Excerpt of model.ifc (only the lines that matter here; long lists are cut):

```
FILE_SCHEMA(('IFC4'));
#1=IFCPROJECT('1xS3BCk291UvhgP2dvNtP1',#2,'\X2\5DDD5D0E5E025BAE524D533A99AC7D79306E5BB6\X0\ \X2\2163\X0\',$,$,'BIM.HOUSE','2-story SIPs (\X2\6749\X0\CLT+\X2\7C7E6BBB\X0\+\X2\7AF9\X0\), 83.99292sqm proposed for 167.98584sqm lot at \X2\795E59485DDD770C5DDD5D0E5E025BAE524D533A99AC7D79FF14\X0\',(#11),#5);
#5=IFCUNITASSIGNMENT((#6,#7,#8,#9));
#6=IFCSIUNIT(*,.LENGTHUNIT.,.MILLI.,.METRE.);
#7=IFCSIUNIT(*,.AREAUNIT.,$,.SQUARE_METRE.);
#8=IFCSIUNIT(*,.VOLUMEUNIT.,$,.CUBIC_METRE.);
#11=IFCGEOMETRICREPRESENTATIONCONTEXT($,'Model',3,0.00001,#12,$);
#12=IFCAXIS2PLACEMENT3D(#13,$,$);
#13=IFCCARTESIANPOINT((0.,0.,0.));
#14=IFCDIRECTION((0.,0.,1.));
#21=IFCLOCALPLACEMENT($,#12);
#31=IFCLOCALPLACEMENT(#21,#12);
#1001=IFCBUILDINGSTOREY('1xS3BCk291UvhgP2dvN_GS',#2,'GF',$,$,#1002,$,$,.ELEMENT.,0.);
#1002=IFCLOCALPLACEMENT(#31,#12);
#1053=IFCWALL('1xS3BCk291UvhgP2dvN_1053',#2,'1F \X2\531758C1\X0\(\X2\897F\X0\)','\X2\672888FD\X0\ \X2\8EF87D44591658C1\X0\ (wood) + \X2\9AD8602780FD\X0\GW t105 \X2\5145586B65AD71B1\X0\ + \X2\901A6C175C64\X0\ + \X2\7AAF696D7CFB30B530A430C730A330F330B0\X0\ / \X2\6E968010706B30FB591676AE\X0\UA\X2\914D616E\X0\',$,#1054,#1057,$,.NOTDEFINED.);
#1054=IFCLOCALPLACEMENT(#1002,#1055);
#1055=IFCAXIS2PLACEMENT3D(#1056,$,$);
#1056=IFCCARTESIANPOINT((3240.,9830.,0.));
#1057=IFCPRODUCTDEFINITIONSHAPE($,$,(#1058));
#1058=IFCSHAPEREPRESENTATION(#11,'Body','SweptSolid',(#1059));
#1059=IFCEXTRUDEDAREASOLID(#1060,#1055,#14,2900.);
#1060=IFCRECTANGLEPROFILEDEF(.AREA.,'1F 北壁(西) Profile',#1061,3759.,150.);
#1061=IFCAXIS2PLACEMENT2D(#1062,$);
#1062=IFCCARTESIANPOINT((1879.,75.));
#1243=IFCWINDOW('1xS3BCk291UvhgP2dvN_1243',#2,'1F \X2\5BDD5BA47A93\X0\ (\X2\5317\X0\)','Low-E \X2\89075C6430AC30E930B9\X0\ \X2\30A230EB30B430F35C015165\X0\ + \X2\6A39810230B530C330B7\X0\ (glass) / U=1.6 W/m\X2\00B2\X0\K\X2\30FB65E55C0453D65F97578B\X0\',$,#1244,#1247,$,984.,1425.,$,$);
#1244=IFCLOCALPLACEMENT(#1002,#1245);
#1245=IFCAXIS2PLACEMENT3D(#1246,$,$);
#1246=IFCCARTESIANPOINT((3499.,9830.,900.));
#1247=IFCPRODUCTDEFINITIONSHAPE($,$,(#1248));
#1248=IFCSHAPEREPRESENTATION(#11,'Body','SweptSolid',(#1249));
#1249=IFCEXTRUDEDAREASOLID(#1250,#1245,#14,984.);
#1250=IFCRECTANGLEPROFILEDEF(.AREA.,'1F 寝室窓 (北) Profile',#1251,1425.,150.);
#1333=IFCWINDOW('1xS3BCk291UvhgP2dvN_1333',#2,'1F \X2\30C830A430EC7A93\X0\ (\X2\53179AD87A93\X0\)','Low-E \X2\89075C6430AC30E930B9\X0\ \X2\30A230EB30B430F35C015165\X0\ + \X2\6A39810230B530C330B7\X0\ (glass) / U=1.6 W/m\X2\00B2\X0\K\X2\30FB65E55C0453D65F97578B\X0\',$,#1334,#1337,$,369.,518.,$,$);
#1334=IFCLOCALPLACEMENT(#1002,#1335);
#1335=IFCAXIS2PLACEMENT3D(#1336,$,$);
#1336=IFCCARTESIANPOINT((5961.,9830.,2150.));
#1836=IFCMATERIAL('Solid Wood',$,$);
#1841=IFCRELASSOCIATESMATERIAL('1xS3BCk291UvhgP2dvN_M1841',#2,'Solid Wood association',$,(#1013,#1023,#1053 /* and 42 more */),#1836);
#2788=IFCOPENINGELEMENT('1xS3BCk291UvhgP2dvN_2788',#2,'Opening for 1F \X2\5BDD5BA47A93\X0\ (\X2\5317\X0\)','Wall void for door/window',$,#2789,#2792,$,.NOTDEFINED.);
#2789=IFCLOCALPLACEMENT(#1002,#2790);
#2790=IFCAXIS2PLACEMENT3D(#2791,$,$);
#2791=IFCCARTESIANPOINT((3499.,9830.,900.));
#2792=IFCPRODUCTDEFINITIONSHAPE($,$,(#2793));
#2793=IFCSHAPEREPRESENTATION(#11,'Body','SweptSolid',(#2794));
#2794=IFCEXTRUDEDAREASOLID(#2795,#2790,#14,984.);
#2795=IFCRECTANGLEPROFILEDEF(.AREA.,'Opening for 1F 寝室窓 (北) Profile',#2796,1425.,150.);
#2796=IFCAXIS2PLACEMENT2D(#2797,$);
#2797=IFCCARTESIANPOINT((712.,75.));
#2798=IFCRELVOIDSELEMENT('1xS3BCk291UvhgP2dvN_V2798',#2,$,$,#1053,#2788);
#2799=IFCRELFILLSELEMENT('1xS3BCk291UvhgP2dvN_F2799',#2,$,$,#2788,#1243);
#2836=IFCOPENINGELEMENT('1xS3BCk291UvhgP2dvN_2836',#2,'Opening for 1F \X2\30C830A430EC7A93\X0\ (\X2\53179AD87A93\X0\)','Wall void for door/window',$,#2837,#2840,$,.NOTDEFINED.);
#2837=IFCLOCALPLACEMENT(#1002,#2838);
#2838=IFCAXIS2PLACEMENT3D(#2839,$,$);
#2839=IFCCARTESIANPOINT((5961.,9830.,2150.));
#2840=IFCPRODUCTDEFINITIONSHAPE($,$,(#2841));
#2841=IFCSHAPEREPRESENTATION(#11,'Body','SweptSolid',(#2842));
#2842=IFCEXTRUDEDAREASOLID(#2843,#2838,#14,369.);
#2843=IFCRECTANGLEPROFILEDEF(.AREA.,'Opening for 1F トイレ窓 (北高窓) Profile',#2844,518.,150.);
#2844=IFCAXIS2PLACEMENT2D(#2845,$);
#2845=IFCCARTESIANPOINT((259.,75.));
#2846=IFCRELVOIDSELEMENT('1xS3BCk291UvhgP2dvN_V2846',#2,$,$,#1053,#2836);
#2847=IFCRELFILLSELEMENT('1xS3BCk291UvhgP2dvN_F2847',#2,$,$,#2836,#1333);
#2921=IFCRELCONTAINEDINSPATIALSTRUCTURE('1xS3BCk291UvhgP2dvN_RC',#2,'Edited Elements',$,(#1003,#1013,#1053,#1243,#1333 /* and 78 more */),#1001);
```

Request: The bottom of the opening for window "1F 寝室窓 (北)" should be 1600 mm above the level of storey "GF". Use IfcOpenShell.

```python
import numpy as np
import ifcopenshell
import ifcopenshell.api.geometry
import ifcopenshell.geom
import ifcopenshell.util.element
import ifcopenshell.util.placement
import ifcopenshell.util.shape
import ifcopenshell.util.unit

model = ifcopenshell.open("model.ifc")
unit_scale = ifcopenshell.util.unit.calculate_unit_scale(model)

window = model.by_guid("1xS3BCk291UvhgP2dvN_1243")
opening = window.FillsVoids[0].RelatingOpeningElement
storey = ifcopenshell.util.element.get_container(window, ifc_class="IfcBuildingStorey")
level = ifcopenshell.util.placement.get_local_placement(storey.ObjectPlacement)[2, 3]

# The opening's origin need not be at the sill, so measure its lowest point.
shape = ifcopenshell.geom.create_shape(ifcopenshell.geom.settings(), opening)
bottom = ifcopenshell.util.shape.get_shape_bottom_elevation(shape, shape.geometry) / unit_scale
dz = level + 1600.0 - bottom

shift = np.array([0.0, 0.0, dz])
# The window is not placed relative to its opening, so move both.
for product in (opening, window):
    matrix = ifcopenshell.util.placement.get_local_placement(product.ObjectPlacement)
    matrix[:3, 3] += shift
    ifcopenshell.api.geometry.edit_object_placement(model, product=product, matrix=matrix, is_si=False)

print(f"moved by {dz * unit_scale:+.3f} m")

model.write("model_v2.ifc")
```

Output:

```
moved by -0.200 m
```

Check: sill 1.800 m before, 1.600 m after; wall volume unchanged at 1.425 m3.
